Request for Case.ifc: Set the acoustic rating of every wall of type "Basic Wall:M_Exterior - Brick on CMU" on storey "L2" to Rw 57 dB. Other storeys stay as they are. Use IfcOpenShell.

First a look at what the model holds.

```python
import ifcopenshell
import ifcopenshell.util.element

model = ifcopenshell.open("Case.ifc")
print(model.schema)
storey = next(s for s in model.by_type("IfcBuildingStorey") if s.Name == "L2")
walls = [e for e in ifcopenshell.util.element.get_decomposition(storey) if e.is_a("IfcWall")]
seen = {}
for e in walls:
    element_type = ifcopenshell.util.element.get_type(e)
    key = (element_type.Name if element_type != e and element_type else None, ifcopenshell.util.element.get_pset(e, "Pset_WallCommon", "AcousticRating"))
    seen[key] = seen.get(key, 0) + 1
for (name, value), count in sorted(seen.items(), key=str):
    print(count, "x", name, "|", value)
```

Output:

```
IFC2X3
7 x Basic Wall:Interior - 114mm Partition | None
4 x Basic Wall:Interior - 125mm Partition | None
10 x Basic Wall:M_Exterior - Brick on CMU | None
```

```python
import ifcopenshell
import ifcopenshell.api.pset
import ifcopenshell.util.element

model = ifcopenshell.open("Case.ifc")

storey = next(s for s in model.by_type("IfcBuildingStorey") if s.Name == "L2")
walls = [e for e in ifcopenshell.util.element.get_decomposition(storey) if e.is_a("IfcWall")]

count = 0
for e in walls:
    element_type = ifcopenshell.util.element.get_type(e)
    if element_type in (None, e) or element_type.Name != "Basic Wall:M_Exterior - Brick on CMU":
        continue
    # add_pset returns the element's existing set when there is one.
    pset = ifcopenshell.api.pset.add_pset(model, product=e, name="Pset_WallCommon")
    ifcopenshell.api.pset.edit_pset(model, pset=pset, properties={"AcousticRating": "Rw 57 dB"})
    count += 1

print(count, "walls updated")

model.write("Case_edited.ifc")
```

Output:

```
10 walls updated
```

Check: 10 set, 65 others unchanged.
